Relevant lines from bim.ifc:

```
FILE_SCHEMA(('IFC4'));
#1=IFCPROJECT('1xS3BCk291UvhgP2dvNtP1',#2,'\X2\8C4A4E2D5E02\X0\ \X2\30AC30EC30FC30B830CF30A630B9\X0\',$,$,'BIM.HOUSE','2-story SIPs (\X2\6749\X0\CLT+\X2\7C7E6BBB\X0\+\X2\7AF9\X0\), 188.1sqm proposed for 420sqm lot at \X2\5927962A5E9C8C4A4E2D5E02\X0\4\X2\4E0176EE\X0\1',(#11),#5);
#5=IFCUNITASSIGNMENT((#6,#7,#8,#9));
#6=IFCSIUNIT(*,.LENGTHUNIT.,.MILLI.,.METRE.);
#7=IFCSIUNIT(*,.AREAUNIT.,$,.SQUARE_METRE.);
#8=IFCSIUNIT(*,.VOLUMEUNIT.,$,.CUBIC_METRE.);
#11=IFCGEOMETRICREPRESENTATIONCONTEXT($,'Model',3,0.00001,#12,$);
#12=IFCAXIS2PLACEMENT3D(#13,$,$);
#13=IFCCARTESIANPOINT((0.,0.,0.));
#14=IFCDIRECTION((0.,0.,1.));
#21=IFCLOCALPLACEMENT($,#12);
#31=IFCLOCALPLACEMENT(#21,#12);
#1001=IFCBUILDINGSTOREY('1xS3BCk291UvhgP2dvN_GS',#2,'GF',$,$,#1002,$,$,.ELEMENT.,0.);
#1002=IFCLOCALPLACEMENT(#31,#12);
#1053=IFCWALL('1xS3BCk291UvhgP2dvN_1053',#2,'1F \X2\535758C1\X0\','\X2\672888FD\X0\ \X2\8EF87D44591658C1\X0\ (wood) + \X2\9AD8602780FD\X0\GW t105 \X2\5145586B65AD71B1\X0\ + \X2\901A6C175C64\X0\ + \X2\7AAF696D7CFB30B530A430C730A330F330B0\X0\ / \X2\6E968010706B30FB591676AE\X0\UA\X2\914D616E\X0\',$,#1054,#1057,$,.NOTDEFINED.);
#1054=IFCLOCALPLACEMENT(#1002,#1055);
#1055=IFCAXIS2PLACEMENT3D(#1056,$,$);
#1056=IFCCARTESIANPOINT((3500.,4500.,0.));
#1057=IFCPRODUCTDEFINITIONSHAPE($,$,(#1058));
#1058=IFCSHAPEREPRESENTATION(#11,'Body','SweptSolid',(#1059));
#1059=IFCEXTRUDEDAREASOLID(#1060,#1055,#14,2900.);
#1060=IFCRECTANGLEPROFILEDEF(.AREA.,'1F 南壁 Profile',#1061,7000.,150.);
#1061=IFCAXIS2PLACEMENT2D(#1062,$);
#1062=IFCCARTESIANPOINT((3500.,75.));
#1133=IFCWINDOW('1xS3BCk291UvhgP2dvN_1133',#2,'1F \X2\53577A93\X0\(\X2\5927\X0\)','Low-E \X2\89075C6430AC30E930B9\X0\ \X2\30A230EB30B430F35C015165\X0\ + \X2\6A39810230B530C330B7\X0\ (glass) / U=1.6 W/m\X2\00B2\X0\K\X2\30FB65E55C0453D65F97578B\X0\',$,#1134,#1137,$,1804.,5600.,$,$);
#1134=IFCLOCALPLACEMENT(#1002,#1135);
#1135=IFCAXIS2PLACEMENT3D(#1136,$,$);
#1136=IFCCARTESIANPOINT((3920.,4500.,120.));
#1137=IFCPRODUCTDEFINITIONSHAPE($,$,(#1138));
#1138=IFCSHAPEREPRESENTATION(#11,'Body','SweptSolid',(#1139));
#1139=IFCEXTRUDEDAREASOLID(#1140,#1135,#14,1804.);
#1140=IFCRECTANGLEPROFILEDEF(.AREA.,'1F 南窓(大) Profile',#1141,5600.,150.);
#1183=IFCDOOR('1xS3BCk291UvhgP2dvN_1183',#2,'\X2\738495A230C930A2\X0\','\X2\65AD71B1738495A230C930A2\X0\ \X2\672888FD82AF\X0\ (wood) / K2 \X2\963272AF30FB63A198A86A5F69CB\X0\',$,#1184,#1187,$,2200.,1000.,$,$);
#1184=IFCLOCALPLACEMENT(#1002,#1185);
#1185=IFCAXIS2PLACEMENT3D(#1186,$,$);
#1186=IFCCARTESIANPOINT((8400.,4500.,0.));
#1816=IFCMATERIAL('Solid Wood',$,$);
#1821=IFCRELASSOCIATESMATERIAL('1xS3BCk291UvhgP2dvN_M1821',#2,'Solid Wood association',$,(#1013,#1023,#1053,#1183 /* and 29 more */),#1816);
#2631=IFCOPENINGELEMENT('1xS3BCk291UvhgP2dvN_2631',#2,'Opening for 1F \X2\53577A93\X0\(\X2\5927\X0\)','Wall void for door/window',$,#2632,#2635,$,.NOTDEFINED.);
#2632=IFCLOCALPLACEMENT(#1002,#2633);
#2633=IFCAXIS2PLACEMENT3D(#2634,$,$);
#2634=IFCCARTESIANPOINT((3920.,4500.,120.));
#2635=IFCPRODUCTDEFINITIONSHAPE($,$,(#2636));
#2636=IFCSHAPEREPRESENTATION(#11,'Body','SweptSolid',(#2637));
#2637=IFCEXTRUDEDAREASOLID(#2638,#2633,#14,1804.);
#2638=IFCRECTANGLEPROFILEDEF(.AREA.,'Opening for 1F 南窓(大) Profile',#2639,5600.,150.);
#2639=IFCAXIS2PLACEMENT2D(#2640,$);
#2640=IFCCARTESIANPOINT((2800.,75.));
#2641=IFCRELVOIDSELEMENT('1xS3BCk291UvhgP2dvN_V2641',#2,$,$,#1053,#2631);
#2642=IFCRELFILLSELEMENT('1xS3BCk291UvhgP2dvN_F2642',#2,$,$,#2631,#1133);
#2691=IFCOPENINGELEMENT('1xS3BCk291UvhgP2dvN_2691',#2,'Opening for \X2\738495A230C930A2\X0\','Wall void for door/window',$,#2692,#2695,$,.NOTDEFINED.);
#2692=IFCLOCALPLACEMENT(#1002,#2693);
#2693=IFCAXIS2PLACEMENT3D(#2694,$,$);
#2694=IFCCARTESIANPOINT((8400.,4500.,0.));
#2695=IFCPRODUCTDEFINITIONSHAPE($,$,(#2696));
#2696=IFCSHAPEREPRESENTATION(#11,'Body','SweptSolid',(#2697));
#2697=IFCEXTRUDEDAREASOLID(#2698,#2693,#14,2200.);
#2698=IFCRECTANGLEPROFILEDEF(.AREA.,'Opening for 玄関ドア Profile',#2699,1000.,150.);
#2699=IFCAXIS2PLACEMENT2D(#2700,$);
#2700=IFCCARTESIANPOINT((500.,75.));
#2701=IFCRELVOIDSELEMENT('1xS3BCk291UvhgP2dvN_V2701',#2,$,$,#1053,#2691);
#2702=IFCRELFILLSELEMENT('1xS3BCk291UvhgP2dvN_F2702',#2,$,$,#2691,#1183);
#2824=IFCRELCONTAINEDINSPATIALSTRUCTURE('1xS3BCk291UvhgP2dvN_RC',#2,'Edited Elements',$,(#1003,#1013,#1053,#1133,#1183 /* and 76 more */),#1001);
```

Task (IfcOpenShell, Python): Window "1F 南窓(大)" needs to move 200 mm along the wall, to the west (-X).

```python
import ifcopenshell
import ifcopenshell.api.geometry
import ifcopenshell.util.placement
import ifcopenshell.util.unit

model = ifcopenshell.open("bim.ifc")
unit_scale = ifcopenshell.util.unit.calculate_unit_scale(model)

window = model.by_guid("1xS3BCk291UvhgP2dvN_1133")
opening = window.FillsVoids[0].RelatingOpeningElement
wall = opening.VoidsElements[0].RelatingBuildingElement

wall_matrix = ifcopenshell.util.placement.get_local_placement(wall.ObjectPlacement)
shift = wall_matrix[:3, 0] * -0.2 / unit_scale
before = ifcopenshell.util.placement.get_local_placement(window.ObjectPlacement)[:3, 3].copy()

# The window is not placed relative to its opening, so move both.
for product in (opening, window):
    matrix = ifcopenshell.util.placement.get_local_placement(product.ObjectPlacement)
    matrix[:3, 3] += shift
    ifcopenshell.api.geometry.edit_object_placement(model, product=product, matrix=matrix, is_si=False)

after = ifcopenshell.util.placement.get_local_placement(window.ObjectPlacement)[:3, 3]
print("window moved by", (after - before).round(3) + 0.0)

model.write("bim_rev.ifc")
```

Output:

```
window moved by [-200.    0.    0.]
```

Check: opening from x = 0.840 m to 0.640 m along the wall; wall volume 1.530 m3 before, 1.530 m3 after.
